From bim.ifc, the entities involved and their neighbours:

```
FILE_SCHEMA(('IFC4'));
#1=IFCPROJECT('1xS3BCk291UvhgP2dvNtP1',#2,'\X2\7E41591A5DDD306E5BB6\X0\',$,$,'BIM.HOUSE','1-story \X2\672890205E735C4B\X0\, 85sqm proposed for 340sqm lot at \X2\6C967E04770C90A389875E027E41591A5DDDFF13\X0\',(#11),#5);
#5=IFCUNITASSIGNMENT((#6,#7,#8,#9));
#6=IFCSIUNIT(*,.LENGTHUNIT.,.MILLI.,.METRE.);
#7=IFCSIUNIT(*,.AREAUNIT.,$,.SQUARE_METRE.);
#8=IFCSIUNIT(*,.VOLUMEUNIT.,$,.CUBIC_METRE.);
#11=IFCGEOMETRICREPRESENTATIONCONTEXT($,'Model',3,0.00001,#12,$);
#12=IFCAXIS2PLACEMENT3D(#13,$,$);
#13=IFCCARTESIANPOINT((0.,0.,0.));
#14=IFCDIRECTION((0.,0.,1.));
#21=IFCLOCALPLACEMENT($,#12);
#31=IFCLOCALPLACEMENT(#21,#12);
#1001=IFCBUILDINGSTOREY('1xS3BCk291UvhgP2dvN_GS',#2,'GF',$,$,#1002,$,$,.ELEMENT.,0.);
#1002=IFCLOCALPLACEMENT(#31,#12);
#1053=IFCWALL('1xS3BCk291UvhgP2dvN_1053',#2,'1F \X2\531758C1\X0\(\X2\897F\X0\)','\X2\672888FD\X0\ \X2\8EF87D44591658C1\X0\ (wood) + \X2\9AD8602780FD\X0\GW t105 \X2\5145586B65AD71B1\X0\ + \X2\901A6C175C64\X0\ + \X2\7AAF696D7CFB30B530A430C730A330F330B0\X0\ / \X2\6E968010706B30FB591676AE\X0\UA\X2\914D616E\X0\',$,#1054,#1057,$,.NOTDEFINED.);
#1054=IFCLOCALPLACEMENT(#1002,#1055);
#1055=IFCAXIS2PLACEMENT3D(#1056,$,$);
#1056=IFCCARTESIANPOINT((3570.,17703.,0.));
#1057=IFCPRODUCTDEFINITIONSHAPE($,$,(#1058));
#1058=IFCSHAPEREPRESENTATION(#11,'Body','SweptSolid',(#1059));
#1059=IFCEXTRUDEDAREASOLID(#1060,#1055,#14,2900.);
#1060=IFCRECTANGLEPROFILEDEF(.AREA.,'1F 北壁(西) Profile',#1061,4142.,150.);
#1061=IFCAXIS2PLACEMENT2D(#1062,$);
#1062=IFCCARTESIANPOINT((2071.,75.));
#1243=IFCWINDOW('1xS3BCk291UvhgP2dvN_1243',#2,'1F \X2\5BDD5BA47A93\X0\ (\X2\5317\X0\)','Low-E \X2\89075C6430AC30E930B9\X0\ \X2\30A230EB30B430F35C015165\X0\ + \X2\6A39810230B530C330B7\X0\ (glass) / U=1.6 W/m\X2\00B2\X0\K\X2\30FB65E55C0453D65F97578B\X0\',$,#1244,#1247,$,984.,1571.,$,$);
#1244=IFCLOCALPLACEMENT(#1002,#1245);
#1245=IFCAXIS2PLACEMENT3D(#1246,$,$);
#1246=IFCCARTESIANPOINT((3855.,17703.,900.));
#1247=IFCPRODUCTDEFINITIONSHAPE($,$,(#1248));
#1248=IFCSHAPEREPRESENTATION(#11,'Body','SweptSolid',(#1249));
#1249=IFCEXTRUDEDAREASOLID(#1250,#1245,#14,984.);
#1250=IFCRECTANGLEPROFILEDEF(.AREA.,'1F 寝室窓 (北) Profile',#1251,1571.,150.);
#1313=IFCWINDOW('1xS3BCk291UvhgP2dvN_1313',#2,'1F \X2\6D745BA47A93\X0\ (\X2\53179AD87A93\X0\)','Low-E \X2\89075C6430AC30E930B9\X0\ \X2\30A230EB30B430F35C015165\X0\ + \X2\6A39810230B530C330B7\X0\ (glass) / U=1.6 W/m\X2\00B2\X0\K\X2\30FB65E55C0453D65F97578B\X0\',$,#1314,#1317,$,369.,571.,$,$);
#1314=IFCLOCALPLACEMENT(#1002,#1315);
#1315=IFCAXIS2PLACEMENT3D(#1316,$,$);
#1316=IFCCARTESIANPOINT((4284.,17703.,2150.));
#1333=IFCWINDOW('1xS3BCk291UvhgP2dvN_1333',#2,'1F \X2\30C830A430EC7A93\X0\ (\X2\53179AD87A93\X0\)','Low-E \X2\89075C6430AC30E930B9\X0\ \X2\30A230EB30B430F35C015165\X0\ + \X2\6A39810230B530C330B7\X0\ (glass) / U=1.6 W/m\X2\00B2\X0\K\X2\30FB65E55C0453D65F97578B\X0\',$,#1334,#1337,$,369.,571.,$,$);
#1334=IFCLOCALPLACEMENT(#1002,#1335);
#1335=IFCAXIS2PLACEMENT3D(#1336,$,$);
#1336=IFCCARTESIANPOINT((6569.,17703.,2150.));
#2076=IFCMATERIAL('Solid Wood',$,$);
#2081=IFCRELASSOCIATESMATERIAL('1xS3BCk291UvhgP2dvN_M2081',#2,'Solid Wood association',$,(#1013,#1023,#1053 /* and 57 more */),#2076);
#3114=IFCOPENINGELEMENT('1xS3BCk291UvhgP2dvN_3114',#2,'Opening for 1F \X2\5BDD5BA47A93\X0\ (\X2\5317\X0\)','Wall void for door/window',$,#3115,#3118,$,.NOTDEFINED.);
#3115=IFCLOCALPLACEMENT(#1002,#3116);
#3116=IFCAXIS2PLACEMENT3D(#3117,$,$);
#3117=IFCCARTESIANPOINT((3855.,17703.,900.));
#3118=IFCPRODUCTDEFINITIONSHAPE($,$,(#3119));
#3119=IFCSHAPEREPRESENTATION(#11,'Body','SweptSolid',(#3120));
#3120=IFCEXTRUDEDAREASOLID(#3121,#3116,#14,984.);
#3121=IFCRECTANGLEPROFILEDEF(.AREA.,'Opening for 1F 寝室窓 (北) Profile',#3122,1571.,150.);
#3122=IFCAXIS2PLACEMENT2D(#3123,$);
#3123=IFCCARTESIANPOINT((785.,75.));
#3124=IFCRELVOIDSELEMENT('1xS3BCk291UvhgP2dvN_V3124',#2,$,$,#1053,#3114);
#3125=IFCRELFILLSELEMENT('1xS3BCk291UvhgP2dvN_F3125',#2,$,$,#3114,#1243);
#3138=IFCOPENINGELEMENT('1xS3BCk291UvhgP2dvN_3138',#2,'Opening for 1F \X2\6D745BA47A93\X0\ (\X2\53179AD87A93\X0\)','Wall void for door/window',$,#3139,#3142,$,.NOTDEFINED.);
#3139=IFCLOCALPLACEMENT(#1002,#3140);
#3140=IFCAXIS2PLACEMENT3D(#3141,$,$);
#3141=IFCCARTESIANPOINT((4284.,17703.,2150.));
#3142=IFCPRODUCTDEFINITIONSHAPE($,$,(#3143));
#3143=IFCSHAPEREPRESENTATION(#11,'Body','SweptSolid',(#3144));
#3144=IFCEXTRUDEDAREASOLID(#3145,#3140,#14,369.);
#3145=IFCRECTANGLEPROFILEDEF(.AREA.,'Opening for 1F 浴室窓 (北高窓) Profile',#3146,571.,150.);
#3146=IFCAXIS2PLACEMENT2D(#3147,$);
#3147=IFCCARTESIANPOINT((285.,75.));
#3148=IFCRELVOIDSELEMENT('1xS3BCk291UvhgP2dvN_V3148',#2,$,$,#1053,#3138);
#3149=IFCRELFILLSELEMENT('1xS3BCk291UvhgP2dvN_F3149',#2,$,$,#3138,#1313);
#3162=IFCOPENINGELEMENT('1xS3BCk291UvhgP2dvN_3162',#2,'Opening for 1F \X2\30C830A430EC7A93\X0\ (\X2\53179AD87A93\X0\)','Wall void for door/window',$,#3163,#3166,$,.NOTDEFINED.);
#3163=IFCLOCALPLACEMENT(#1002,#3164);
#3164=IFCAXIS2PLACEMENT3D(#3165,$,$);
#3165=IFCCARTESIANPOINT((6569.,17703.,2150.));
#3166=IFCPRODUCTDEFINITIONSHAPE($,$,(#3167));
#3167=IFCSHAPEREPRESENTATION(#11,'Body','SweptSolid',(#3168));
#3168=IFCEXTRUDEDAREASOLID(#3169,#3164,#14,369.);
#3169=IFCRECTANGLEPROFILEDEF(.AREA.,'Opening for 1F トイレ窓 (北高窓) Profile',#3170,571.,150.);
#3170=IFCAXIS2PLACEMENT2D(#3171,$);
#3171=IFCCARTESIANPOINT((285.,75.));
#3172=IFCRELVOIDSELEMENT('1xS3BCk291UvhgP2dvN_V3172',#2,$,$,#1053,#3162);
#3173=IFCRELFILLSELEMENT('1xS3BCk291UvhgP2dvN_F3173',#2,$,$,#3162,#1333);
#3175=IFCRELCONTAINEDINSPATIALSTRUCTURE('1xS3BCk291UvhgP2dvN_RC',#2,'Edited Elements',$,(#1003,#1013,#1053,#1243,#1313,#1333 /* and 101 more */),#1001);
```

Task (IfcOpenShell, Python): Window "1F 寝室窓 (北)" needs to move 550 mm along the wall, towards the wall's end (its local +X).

```python
import ifcopenshell
import ifcopenshell.api.geometry
import ifcopenshell.util.placement

model = ifcopenshell.open("bim.ifc")

window = model.by_id(1243)
opening = window.FillsVoids[0].RelatingOpeningElement
wall = opening.VoidsElements[0].RelatingBuildingElement

wall_matrix = ifcopenshell.util.placement.get_local_placement(wall.ObjectPlacement)
shift = wall_matrix[:3, 0] * 550.0
before = ifcopenshell.util.placement.get_local_placement(window.ObjectPlacement)[:3, 3].copy()

# The window is not placed relative to its opening, so move both.
for product in (opening, window):
    matrix = ifcopenshell.util.placement.get_local_placement(product.ObjectPlacement)
    matrix[:3, 3] += shift
    ifcopenshell.api.geometry.edit_object_placement(model, product=product, matrix=matrix, is_si=False)

after = ifcopenshell.util.placement.get_local_placement(window.ObjectPlacement)[:3, 3]
print("window moved by", (after - before).round(3) + 0.0)

model.write("bim-out.ifc")
```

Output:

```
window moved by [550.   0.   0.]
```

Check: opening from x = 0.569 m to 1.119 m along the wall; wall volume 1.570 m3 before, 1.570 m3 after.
